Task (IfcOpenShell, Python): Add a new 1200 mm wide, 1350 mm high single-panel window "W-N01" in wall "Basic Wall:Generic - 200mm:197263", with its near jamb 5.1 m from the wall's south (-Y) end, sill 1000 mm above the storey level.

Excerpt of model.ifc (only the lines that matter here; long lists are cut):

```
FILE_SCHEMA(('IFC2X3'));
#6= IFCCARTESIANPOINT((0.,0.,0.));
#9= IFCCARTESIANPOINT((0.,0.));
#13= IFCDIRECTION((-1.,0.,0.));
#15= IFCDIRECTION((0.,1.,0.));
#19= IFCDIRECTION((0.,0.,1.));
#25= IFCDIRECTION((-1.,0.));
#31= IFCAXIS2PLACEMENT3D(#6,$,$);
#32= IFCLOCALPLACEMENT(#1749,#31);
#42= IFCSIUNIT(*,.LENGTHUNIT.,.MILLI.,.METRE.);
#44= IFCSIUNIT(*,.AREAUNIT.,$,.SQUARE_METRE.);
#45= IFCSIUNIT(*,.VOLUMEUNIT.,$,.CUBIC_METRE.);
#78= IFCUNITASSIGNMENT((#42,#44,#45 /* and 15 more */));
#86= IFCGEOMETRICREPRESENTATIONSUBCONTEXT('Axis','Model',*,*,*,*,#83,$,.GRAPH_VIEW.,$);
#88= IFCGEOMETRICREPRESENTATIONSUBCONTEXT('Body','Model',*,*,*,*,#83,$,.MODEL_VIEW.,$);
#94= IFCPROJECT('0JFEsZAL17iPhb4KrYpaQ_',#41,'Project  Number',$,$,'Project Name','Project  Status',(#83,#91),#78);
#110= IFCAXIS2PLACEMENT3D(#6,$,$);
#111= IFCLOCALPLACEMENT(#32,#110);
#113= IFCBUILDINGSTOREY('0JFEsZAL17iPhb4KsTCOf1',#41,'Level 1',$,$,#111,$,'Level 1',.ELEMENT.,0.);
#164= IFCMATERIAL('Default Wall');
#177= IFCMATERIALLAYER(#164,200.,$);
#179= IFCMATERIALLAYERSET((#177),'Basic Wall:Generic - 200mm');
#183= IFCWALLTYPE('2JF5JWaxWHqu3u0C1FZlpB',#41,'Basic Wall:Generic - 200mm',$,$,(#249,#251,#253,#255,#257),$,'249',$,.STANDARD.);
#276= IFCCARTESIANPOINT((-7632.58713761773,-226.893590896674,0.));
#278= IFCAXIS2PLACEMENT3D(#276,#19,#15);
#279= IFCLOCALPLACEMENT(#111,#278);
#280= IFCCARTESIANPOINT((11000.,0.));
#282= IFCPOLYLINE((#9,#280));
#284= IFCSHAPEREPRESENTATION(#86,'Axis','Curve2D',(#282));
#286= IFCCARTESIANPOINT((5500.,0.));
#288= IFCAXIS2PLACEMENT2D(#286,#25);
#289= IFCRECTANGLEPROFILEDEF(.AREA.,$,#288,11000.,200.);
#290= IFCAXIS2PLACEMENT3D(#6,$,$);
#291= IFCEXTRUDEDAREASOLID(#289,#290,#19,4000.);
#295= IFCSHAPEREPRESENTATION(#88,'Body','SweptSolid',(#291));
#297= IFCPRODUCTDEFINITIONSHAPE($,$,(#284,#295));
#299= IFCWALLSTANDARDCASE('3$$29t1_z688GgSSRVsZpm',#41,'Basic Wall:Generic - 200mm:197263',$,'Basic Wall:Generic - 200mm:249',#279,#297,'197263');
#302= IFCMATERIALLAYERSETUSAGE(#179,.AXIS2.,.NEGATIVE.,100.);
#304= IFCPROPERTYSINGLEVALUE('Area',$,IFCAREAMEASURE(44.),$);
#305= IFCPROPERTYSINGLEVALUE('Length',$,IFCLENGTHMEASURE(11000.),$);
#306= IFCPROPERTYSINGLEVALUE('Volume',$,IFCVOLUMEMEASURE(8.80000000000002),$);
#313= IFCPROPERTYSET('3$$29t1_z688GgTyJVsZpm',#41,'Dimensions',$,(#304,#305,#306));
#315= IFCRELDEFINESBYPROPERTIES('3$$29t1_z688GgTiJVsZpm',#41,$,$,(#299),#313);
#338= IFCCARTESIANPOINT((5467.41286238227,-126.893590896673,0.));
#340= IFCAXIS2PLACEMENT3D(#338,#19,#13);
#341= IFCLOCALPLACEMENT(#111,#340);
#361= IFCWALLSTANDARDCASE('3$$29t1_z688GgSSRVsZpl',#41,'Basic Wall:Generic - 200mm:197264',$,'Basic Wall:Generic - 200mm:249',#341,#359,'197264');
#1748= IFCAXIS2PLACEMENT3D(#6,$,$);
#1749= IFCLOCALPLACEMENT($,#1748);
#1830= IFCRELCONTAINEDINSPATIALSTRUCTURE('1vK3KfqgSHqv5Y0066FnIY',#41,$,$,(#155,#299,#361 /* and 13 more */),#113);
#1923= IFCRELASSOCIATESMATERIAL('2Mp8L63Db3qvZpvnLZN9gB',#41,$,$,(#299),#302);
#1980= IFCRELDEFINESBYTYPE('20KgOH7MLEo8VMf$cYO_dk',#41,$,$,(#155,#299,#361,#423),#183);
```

```python
import numpy as np
import ifcopenshell
import ifcopenshell.api.feature
import ifcopenshell.api.geometry
import ifcopenshell.api.pset
import ifcopenshell.api.root
import ifcopenshell.api.spatial
import ifcopenshell.api.type
import ifcopenshell.geom
import ifcopenshell.util.element
import ifcopenshell.util.placement
import ifcopenshell.util.representation
import ifcopenshell.util.shape
import ifcopenshell.util.unit

model = ifcopenshell.open("model.ifc")
unit_scale = ifcopenshell.util.unit.calculate_unit_scale(model)
area_scale = ifcopenshell.util.unit.calculate_unit_scale(model, "AREAUNIT")
volume_scale = ifcopenshell.util.unit.calculate_unit_scale(model, "VOLUMEUNIT")
settings = ifcopenshell.geom.settings()


def volume(element):
    """Net volume in cubic metres, openings subtracted."""
    shape = ifcopenshell.geom.create_shape(settings, element)
    return ifcopenshell.util.shape.get_volume(shape.geometry)


wall = model.by_guid("3$$29t1_z688GgSSRVsZpm")
storey = ifcopenshell.util.element.get_container(wall, ifc_class="IfcBuildingStorey")
context = ifcopenshell.util.representation.get_context(model, "Model", "Body", "MODEL_VIEW")
before = volume(wall)

width, height, from_end, sill = 1.2, 1.35, 5.1, 1  # metres

# The wall runs along its own X axis, and the end named is its -X end.
wall_shape = ifcopenshell.geom.create_shape(settings, wall)
x, y, z = ifcopenshell.util.shape.get_vertices(wall_shape.geometry).T
start = x.min() + from_end
face, thickness = float(y.min()), float(y.max() - y.min())
wall_matrix = ifcopenshell.util.placement.get_local_placement(wall.ObjectPlacement)
level = ifcopenshell.util.placement.get_local_placement(storey.ObjectPlacement)[2, 3]


def in_wall(x, y):
    """Placement at x, y metres in the wall's axes, at sill height."""
    matrix = wall_matrix.copy()
    matrix[:, 3] = wall_matrix @ np.array([x / unit_scale, y / unit_scale, 0.0, 1.0])
    matrix[2, 3] = level + sill / unit_scale
    return matrix


# Opening: a box that overshoots both wall faces by 50 mm.
opening = ifcopenshell.api.root.create_entity(model, ifc_class="IfcOpeningElement")
box = ifcopenshell.api.geometry.add_wall_representation(
    model, context=context, length=width, height=height, thickness=thickness + 0.1
)
ifcopenshell.api.geometry.assign_representation(model, product=opening, representation=box)
ifcopenshell.api.geometry.edit_object_placement(model, product=opening, matrix=in_wall(start, face - 0.05), is_si=False)
ifcopenshell.api.feature.add_feature(model, feature=opening, element=wall)

window = ifcopenshell.api.root.create_entity(model, ifc_class="IfcWindow", name="W-N01")
window.OverallWidth, window.OverallHeight = width / unit_scale, height / unit_scale
body = ifcopenshell.api.geometry.add_window_representation(
    model,
    context=context,
    overall_width=window.OverallWidth,
    overall_height=window.OverallHeight,
    partition_type="SINGLE_PANEL",
)
ifcopenshell.api.geometry.assign_representation(model, product=window, representation=body)
ifcopenshell.api.spatial.assign_container(model, products=[window], relating_structure=storey)
fills = ifcopenshell.api.feature.add_filling(model, opening=opening, element=window)
fills.OwnerHistory = window.OwnerHistory  # required in IFC2X3

# IFC2X3 keeps the operation on the window style.
style = ifcopenshell.api.root.create_entity(model, ifc_class="IfcWindowStyle", name="W-N01")
style.OperationType, style.ConstructionType = "SINGLE_PANEL", "NOTDEFINED"
style.ParameterTakesPrecedence = style.Sizeable = False
ifcopenshell.api.type.assign_type(model, related_objects=[window], relating_type=style)

# Centre the window in the wall's thickness.
ifcopenshell.api.geometry.edit_object_placement(model, product=window, matrix=in_wall(start, face), is_si=False)
window_shape = ifcopenshell.geom.create_shape(settings, window)
depth = ifcopenshell.util.shape.get_vertices(window_shape.geometry)[:, 1]
offset = face + thickness / 2 - (depth.min() + depth.max()) / 2
ifcopenshell.api.geometry.edit_object_placement(model, product=window, matrix=in_wall(start, offset), is_si=False)

after = volume(wall)

# Update the wall's stored quantities.
pset = model.by_id(ifcopenshell.util.element.get_pset(wall, "Dimensions", should_inherit=False)["id"])
ifcopenshell.api.pset.edit_pset(model, pset=pset, properties={
    "Area": model.create_entity("IfcAreaMeasure", after / thickness / area_scale),
    "Volume": model.create_entity("IfcVolumeMeasure", after / volume_scale),
})

print(f"wall volume {before:.3f} -> {after:.3f} m3")

model.write("model_updated.ifc")
```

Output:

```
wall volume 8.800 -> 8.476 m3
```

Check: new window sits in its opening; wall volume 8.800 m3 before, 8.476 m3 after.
